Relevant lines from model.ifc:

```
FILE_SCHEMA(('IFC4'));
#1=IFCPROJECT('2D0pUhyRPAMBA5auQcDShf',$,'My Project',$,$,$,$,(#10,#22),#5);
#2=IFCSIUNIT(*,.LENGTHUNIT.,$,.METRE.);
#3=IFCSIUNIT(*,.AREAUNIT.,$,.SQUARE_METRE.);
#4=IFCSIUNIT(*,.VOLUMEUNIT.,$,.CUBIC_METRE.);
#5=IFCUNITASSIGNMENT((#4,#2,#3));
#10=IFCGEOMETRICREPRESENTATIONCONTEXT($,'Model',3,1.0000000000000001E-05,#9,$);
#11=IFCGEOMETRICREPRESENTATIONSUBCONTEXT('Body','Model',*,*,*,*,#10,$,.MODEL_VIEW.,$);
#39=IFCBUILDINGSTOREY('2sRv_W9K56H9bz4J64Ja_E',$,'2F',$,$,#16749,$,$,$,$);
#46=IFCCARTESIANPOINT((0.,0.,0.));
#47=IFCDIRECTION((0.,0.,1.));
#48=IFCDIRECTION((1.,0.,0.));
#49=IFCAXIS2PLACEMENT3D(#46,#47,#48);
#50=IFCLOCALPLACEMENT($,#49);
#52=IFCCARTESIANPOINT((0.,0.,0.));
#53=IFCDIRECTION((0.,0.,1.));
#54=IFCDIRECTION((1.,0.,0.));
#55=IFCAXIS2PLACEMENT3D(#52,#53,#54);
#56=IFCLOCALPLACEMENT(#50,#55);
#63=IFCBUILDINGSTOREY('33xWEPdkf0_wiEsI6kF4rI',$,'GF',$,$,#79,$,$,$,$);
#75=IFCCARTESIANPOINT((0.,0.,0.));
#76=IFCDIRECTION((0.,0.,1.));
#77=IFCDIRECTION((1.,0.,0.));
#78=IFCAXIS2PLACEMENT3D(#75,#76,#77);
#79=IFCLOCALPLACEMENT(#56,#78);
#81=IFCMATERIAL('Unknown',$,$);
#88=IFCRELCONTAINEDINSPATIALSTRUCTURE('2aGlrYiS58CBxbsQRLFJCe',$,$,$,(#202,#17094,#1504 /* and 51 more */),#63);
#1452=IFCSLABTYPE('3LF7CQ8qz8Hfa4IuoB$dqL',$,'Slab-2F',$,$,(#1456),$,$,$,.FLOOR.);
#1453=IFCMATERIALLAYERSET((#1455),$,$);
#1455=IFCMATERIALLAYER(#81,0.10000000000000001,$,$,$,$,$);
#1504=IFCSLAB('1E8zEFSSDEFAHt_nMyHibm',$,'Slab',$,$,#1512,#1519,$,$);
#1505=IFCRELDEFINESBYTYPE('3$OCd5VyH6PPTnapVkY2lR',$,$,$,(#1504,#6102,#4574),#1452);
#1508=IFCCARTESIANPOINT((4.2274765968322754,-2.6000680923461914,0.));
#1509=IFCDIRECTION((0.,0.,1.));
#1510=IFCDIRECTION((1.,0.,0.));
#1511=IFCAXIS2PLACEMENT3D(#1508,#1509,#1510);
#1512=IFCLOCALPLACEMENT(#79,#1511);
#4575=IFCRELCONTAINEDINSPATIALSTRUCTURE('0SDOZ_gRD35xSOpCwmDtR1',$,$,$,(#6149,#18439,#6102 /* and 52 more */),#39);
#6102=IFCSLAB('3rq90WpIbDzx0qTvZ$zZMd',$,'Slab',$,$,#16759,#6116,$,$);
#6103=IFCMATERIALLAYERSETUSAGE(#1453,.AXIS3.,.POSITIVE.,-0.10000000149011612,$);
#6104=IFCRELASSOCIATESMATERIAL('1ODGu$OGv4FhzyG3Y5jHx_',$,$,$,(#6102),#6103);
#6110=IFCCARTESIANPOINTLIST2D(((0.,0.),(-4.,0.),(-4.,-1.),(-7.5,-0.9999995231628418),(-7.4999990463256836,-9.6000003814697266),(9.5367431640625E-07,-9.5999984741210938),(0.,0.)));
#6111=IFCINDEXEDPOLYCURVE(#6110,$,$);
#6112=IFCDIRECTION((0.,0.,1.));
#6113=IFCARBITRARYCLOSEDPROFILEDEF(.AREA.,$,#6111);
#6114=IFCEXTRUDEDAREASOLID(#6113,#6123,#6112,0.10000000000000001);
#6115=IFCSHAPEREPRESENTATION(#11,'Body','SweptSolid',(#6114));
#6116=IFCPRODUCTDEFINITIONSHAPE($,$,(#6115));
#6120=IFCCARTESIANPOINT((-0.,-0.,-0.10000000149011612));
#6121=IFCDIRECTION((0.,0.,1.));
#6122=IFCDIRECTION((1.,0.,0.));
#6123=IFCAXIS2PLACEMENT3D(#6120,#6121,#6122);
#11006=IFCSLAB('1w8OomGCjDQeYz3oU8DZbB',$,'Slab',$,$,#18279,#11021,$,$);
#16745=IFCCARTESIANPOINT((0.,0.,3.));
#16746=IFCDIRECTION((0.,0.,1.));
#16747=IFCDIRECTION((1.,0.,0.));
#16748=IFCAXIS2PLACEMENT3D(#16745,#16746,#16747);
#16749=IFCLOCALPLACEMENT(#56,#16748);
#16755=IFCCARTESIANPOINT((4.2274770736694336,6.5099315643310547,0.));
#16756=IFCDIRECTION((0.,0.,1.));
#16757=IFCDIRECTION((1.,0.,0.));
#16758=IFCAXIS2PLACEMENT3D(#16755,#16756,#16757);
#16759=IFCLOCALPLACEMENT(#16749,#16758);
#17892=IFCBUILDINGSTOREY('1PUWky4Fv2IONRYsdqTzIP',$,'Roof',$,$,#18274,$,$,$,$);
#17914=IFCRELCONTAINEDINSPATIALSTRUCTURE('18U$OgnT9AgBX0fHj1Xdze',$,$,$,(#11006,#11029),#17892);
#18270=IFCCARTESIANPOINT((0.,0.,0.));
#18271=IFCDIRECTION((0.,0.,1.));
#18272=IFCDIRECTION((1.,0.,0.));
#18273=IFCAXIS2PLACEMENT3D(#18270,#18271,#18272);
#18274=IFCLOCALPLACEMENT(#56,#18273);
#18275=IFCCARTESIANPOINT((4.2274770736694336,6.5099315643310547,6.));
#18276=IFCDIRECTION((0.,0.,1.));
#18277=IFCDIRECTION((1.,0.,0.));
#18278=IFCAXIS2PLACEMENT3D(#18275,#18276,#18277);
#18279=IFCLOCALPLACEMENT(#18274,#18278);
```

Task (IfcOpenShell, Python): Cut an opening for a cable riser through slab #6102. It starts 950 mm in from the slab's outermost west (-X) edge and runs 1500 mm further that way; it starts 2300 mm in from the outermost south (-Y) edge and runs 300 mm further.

```python
import numpy as np
import ifcopenshell
import ifcopenshell.api.feature
import ifcopenshell.api.geometry
import ifcopenshell.api.root
import ifcopenshell.geom
import ifcopenshell.util.placement
import ifcopenshell.util.representation
import ifcopenshell.util.shape
import ifcopenshell.util.unit

model = ifcopenshell.open("model.ifc")
unit_scale = ifcopenshell.util.unit.calculate_unit_scale(model)
settings = ifcopenshell.geom.settings()


def volume(element):
    """Net volume in cubic metres, openings subtracted."""
    shape = ifcopenshell.geom.create_shape(settings, element)
    return ifcopenshell.util.shape.get_volume(shape.geometry)


slab = model.by_guid("3rq90WpIbDzx0qTvZ$zZMd")
before = volume(slab)

# Extent in the slab's own axes, in metres. The edges named are its -X and -Y sides.
slab_shape = ifcopenshell.geom.create_shape(settings, slab)
vertices = ifcopenshell.util.shape.get_vertices(slab_shape.geometry)
x_min, y_min, bottom = vertices.min(axis=0)
top = vertices[:, 2].max()

opening = ifcopenshell.api.root.create_entity(model, ifc_class="IfcOpeningElement", name="Cable riser opening", predefined_type="OPENING")
context = ifcopenshell.util.representation.get_context(model, "Model", "Body", "MODEL_VIEW")
width, depth = 1.5, 0.3
outline = [(0.0, 0.0), (width, 0.0), (width, depth), (0.0, depth), (0.0, 0.0)]
# Overshoot both faces by 50 mm so the cut is clean.
shape = ifcopenshell.api.geometry.add_slab_representation(
    model, context=context, depth=top - bottom + 0.1, polyline=outline
)
ifcopenshell.api.geometry.assign_representation(model, product=opening, representation=shape)

matrix = ifcopenshell.util.placement.get_local_placement(slab.ObjectPlacement)
matrix[:, 3] = matrix @ np.append(np.array([x_min + 0.95, y_min + 2.3, bottom - 0.05]) / unit_scale, 1.0)
ifcopenshell.api.geometry.edit_object_placement(model, product=opening, matrix=matrix, is_si=False)
ifcopenshell.api.feature.add_feature(model, feature=opening, element=slab)

after = volume(slab)

print(f"slab volume {before:.3f} -> {after:.3f} m3")

model.write("model_edited.ifc")
```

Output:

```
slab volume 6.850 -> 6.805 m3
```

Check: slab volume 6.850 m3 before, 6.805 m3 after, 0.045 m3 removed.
